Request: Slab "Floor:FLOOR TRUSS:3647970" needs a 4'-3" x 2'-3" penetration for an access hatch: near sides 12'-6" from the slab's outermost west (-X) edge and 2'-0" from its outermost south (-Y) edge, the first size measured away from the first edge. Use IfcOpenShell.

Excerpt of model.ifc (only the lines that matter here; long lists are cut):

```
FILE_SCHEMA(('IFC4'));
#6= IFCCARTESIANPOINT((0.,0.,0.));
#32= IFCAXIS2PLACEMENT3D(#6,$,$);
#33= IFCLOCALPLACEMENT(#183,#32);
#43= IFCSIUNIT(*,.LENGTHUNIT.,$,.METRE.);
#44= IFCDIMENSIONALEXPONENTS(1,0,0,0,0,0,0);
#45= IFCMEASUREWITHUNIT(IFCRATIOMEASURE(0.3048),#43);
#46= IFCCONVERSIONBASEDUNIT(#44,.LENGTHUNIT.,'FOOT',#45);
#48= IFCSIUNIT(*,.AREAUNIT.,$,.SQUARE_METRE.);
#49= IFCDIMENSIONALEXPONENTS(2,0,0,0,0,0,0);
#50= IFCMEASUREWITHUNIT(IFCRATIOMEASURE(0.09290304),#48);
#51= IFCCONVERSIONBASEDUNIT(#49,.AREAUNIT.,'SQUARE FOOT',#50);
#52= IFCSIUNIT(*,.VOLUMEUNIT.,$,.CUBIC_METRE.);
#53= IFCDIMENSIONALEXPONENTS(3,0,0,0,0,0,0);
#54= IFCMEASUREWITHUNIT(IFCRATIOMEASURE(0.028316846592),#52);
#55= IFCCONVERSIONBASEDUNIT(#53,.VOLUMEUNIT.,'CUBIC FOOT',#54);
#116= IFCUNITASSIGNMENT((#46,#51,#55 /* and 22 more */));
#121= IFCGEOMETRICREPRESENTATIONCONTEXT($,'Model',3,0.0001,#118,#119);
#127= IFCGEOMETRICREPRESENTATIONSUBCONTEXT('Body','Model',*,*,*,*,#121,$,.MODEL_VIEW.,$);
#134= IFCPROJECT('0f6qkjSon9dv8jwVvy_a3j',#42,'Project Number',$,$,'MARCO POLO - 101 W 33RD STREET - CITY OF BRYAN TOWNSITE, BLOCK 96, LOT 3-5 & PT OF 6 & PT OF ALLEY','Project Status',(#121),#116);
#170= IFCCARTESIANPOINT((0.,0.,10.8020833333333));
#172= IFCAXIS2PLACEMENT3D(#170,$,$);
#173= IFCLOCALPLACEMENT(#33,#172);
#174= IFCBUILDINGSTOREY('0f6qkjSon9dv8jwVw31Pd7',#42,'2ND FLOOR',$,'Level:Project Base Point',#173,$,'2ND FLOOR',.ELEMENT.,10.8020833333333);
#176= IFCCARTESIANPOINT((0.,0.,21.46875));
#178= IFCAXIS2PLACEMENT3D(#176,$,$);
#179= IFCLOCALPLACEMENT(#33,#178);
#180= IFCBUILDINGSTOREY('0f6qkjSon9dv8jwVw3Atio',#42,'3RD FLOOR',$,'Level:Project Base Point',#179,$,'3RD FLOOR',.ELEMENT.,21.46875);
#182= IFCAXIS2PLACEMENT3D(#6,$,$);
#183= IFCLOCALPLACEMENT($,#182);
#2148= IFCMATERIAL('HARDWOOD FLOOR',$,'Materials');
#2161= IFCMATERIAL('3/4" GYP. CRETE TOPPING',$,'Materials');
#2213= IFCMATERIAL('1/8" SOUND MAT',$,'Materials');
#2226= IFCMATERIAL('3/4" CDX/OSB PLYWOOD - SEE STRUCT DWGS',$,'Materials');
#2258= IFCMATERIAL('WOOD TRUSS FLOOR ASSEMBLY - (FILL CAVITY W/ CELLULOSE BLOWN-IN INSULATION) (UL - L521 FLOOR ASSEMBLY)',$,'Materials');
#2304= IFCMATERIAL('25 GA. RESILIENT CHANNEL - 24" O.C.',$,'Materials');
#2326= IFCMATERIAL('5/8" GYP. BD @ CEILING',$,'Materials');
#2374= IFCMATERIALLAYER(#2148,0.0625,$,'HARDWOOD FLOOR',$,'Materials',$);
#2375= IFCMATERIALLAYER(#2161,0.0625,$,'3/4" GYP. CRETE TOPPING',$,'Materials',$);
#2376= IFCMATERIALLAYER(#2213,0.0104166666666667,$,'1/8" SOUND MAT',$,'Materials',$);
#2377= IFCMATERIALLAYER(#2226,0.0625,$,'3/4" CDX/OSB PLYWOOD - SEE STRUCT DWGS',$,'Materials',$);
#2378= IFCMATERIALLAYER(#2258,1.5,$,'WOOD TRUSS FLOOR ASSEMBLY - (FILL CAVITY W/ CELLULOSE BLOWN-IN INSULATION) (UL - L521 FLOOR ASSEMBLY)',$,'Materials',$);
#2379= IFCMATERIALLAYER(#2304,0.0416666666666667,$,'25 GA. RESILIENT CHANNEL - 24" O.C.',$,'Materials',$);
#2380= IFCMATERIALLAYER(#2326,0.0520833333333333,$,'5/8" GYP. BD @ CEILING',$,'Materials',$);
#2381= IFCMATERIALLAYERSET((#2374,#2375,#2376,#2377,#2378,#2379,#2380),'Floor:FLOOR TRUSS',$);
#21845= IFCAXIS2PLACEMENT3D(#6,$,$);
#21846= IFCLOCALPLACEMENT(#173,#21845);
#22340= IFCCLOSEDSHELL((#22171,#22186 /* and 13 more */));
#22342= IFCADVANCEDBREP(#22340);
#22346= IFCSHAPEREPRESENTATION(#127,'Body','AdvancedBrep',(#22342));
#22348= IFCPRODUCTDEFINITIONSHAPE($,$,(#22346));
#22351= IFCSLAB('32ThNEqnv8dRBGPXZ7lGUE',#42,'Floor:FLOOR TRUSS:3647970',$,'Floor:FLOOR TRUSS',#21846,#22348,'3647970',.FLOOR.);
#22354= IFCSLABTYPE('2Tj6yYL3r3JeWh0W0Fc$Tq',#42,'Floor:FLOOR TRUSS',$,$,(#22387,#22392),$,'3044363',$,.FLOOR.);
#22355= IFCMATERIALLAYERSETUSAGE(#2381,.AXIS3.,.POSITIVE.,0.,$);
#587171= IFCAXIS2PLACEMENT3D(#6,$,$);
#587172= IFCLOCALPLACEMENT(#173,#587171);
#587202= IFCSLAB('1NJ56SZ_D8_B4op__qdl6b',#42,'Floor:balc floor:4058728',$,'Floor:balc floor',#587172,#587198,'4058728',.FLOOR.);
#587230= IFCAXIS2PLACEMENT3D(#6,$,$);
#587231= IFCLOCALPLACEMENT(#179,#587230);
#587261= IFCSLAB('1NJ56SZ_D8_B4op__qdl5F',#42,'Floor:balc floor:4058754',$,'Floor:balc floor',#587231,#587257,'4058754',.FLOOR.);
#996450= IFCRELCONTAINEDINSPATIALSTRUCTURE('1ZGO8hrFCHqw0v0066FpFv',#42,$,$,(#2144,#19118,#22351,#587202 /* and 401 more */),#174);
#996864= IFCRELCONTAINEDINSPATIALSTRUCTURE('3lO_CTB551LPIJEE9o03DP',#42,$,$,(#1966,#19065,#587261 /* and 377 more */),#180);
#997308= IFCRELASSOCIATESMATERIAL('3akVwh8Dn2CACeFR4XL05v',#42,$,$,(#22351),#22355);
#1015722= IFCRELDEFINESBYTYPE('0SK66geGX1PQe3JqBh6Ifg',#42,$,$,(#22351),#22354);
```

```python
import numpy as np
import ifcopenshell
import ifcopenshell.api.feature
import ifcopenshell.api.geometry
import ifcopenshell.api.root
import ifcopenshell.geom
import ifcopenshell.util.placement
import ifcopenshell.util.representation
import ifcopenshell.util.shape
import ifcopenshell.util.unit

model = ifcopenshell.open("model.ifc")
unit_scale = ifcopenshell.util.unit.calculate_unit_scale(model)
settings = ifcopenshell.geom.settings()


def volume(element):
    """Net volume in cubic metres, openings subtracted."""
    shape = ifcopenshell.geom.create_shape(settings, element)
    return ifcopenshell.util.shape.get_volume(shape.geometry)


slab = model.by_id(22351)
before = volume(slab)

# Extent in the slab's own axes, in metres. The edges named are its -X and -Y sides.
slab_shape = ifcopenshell.geom.create_shape(settings, slab)
vertices = ifcopenshell.util.shape.get_vertices(slab_shape.geometry)
x_min, y_min, bottom = vertices.min(axis=0)
top = vertices[:, 2].max()

opening = ifcopenshell.api.root.create_entity(model, ifc_class="IfcOpeningElement", name="Access hatch opening", predefined_type="OPENING")
context = ifcopenshell.util.representation.get_context(model, "Model", "Body", "MODEL_VIEW")
width, depth = 1.2954, 0.6858
outline = [(0.0, 0.0), (width, 0.0), (width, depth), (0.0, depth), (0.0, 0.0)]
# Overshoot both faces by 50 mm so the cut is clean.
shape = ifcopenshell.api.geometry.add_slab_representation(
    model, context=context, depth=top - bottom + 0.1, polyline=outline
)
ifcopenshell.api.geometry.assign_representation(model, product=opening, representation=shape)

matrix = ifcopenshell.util.placement.get_local_placement(slab.ObjectPlacement)
matrix[:, 3] = matrix @ np.append(np.array([x_min + 3.81, y_min + 0.6096, bottom - 0.05]) / unit_scale, 1.0)
ifcopenshell.api.geometry.edit_object_placement(model, product=opening, matrix=matrix, is_si=False)
ifcopenshell.api.feature.add_feature(model, feature=opening, element=slab)

after = volume(slab)

print(f"slab volume {before:.3f} -> {after:.3f} m3")

model.write("model-out.ifc")
```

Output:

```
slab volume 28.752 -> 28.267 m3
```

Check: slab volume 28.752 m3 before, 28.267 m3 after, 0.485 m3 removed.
